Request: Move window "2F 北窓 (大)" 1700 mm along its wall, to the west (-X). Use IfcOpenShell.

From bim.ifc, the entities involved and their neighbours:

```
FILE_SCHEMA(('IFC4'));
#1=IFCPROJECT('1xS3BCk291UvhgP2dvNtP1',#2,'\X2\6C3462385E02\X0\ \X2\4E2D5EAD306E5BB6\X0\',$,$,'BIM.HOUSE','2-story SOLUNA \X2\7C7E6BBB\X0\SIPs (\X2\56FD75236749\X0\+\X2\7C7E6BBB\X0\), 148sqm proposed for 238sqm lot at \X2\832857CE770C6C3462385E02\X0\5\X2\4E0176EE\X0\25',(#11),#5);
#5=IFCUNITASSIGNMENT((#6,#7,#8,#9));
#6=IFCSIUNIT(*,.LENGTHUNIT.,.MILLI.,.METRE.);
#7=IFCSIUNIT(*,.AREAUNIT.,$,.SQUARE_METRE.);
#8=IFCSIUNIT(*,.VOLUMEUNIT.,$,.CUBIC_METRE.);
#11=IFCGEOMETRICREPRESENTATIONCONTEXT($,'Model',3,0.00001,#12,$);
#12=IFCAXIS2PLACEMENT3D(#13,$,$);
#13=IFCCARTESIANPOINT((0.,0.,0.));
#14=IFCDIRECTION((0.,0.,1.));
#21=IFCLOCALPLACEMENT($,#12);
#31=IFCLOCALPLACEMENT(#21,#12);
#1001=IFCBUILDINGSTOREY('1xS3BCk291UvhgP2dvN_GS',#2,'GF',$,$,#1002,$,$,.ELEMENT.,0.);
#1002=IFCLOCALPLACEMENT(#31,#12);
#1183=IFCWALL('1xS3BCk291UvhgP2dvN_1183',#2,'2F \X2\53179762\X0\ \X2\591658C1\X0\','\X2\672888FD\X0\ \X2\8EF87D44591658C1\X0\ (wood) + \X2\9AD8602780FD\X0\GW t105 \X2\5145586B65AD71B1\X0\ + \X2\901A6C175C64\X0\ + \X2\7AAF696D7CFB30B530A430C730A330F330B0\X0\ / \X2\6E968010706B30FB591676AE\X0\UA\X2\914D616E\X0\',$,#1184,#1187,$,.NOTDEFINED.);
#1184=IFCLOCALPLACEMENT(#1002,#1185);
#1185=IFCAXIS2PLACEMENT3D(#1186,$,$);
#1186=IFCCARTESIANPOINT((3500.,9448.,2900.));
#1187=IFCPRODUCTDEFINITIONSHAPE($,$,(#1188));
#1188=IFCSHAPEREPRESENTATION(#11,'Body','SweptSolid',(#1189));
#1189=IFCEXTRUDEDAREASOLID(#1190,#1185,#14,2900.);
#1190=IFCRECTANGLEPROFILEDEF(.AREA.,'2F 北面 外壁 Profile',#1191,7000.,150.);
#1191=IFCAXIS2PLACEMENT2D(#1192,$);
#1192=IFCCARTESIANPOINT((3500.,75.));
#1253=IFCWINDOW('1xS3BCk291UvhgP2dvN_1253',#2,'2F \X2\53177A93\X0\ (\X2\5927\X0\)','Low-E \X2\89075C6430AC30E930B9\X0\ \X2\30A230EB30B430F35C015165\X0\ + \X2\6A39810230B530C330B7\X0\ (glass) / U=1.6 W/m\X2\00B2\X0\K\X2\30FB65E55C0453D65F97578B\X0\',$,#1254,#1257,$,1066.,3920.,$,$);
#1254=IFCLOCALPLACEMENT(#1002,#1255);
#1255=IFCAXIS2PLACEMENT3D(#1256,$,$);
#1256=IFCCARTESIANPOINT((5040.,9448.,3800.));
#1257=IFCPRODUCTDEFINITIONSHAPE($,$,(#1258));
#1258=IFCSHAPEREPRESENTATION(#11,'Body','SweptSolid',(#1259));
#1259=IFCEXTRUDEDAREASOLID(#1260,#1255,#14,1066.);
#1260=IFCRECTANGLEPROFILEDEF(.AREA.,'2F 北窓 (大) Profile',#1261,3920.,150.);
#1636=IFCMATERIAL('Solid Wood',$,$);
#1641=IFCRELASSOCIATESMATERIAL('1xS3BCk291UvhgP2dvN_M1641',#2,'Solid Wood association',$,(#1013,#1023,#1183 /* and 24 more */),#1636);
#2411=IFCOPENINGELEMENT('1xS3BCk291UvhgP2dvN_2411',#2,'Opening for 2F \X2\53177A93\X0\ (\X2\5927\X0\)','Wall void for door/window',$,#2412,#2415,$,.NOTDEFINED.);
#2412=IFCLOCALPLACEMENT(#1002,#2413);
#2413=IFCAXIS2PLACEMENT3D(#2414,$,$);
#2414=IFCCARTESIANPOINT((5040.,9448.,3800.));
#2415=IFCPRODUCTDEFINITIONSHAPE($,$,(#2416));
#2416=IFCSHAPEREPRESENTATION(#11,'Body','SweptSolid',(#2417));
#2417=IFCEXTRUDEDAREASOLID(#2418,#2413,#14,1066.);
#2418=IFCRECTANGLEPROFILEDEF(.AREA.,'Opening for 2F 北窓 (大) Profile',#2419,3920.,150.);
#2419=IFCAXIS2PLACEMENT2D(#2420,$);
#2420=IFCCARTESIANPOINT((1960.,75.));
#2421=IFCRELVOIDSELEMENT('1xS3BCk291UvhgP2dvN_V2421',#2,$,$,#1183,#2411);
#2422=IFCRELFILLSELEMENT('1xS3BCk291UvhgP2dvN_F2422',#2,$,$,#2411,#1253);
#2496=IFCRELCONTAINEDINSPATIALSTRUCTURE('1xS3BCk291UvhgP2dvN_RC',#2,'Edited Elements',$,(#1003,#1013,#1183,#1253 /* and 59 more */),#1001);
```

```python
import ifcopenshell
import ifcopenshell.api.geometry
import ifcopenshell.util.placement
import ifcopenshell.util.unit

model = ifcopenshell.open("bim.ifc")
unit_scale = ifcopenshell.util.unit.calculate_unit_scale(model)

window = model.by_guid("1xS3BCk291UvhgP2dvN_1253")
opening = window.FillsVoids[0].RelatingOpeningElement
wall = opening.VoidsElements[0].RelatingBuildingElement

wall_matrix = ifcopenshell.util.placement.get_local_placement(wall.ObjectPlacement)
shift = wall_matrix[:3, 0] * -1.7 / unit_scale
before = ifcopenshell.util.placement.get_local_placement(window.ObjectPlacement)[:3, 3].copy()

# The window is not placed relative to its opening, so move both.
for product in (opening, window):
    matrix = ifcopenshell.util.placement.get_local_placement(product.ObjectPlacement)
    matrix[:3, 3] += shift
    ifcopenshell.api.geometry.edit_object_placement(model, product=product, matrix=matrix, is_si=False)

after = ifcopenshell.util.placement.get_local_placement(window.ObjectPlacement)[:3, 3]
print("window moved by", (after - before).round(3) + 0.0)

model.write("bim-out.ifc")
```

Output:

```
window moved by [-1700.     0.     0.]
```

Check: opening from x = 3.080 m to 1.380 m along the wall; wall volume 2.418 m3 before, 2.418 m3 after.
